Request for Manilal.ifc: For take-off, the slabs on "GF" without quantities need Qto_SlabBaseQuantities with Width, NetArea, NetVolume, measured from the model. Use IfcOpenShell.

First a look at what the model holds.

```python
import ifcopenshell
import ifcopenshell.util.element
import ifcopenshell.util.unit

model = ifcopenshell.open("Manilal.ifc")
print(model.schema)
for unit_type in ("LENGTHUNIT", "AREAUNIT", "VOLUMEUNIT"):
    print(unit_type, ifcopenshell.util.unit.calculate_unit_scale(model, unit_type))
storey = next(s for s in model.by_type("IfcBuildingStorey") if s.Name == "GF")
slabs = [e for e in ifcopenshell.util.element.get_decomposition(storey) if e.is_a("IfcSlab")]
for e in sorted(slabs, key=lambda e: e.id()):
    print(e.id(), e.is_a(), e.Name, list(ifcopenshell.util.element.get_psets(e, qtos_only=True)), sep=" | ")
```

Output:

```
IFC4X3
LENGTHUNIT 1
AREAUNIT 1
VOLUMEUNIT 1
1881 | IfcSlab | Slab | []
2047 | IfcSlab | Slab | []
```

```python
import ifcopenshell
import ifcopenshell.api.pset
import ifcopenshell.geom
import ifcopenshell.util.element
import ifcopenshell.util.shape
import ifcopenshell.util.unit

model = ifcopenshell.open("Manilal.ifc")
unit_scale = ifcopenshell.util.unit.calculate_unit_scale(model)
area_scale = ifcopenshell.util.unit.calculate_unit_scale(model, "AREAUNIT")
volume_scale = ifcopenshell.util.unit.calculate_unit_scale(model, "VOLUMEUNIT")
settings = ifcopenshell.geom.settings()

storey = next(s for s in model.by_type("IfcBuildingStorey") if s.Name == "GF")
slabs = [e for e in ifcopenshell.util.element.get_decomposition(storey) if e.is_a("IfcSlab")]

for e in sorted(slabs, key=lambda e: e.id()):
    if ifcopenshell.util.element.get_psets(e, qtos_only=True, should_inherit=False):
        continue
    # Geometry comes back in metres, in the element's own axes.
    shape = ifcopenshell.geom.create_shape(settings, e)
    values = {
        "Width": ifcopenshell.util.shape.get_z(shape.geometry) / unit_scale,
        "NetArea": ifcopenshell.util.shape.get_footprint_area(shape.geometry) / area_scale,
        "NetVolume": ifcopenshell.util.shape.get_volume(shape.geometry) / volume_scale,
    }
    qto = ifcopenshell.api.pset.add_qto(model, product=e, name="Qto_SlabBaseQuantities")
    ifcopenshell.api.pset.edit_qto(model, qto=qto, properties=values)
    print(e.id(), {k: round(v, 3) for k, v in values.items()})

model.write("Manilal_v2.ifc")
```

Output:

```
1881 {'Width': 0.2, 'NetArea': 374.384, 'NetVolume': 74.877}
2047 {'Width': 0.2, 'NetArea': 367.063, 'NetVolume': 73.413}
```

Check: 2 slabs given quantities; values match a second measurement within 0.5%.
